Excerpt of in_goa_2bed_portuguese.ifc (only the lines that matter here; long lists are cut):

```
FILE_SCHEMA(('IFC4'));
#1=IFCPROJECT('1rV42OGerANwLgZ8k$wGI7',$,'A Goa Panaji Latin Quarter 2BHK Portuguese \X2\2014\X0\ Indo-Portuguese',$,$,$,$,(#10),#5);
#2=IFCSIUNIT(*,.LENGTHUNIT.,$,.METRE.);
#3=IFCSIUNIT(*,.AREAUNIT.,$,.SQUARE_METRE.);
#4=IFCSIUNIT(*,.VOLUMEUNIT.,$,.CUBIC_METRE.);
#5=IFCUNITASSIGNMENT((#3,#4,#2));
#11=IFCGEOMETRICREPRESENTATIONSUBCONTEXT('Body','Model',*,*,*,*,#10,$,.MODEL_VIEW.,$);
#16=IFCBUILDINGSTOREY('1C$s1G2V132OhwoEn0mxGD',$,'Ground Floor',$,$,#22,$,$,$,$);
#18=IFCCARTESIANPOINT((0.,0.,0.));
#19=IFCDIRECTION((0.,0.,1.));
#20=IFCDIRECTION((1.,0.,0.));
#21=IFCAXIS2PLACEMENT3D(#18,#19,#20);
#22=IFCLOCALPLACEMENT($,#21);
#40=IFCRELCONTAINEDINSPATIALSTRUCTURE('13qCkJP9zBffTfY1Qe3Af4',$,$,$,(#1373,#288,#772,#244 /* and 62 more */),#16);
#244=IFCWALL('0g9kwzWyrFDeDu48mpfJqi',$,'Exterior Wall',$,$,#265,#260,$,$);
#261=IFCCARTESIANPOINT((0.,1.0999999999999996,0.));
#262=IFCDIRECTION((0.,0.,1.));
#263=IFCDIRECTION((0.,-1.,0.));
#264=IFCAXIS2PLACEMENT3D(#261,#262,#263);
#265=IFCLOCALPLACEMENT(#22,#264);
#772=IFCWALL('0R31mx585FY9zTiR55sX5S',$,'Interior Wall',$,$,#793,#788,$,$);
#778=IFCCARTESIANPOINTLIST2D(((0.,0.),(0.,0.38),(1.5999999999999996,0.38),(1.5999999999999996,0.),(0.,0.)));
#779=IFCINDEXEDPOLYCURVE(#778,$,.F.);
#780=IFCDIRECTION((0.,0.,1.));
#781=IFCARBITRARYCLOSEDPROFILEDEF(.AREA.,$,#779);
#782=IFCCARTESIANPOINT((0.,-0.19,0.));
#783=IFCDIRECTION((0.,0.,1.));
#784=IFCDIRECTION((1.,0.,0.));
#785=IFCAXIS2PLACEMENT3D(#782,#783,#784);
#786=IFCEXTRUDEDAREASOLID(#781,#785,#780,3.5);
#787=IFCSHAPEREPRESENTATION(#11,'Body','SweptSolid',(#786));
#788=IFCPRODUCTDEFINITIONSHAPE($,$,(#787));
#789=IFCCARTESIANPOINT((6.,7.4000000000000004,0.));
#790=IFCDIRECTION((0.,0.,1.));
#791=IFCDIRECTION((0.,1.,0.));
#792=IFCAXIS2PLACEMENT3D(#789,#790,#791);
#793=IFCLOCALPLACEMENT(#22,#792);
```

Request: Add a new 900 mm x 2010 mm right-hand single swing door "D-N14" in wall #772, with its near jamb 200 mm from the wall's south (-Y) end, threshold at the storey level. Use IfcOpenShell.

```python
import numpy as np
import ifcopenshell
import ifcopenshell.api.feature
import ifcopenshell.api.geometry
import ifcopenshell.api.root
import ifcopenshell.api.spatial
import ifcopenshell.geom
import ifcopenshell.util.element
import ifcopenshell.util.placement
import ifcopenshell.util.representation
import ifcopenshell.util.shape
import ifcopenshell.util.unit

model = ifcopenshell.open("in_goa_2bed_portuguese.ifc")
unit_scale = ifcopenshell.util.unit.calculate_unit_scale(model)
settings = ifcopenshell.geom.settings()


def volume(element):
    """Net volume in cubic metres, openings subtracted."""
    shape = ifcopenshell.geom.create_shape(settings, element)
    return ifcopenshell.util.shape.get_volume(shape.geometry)


wall = model.by_id(772)
storey = ifcopenshell.util.element.get_container(wall, ifc_class="IfcBuildingStorey")
context = ifcopenshell.util.representation.get_context(model, "Model", "Body", "MODEL_VIEW")
before = volume(wall)

width, height, from_end, sill = 0.9, 2.01, 0.2, 0.0  # metres

# The wall runs along its own X axis, and the end named is its -X end.
wall_shape = ifcopenshell.geom.create_shape(settings, wall)
x, y, z = ifcopenshell.util.shape.get_vertices(wall_shape.geometry).T
start = x.min() + from_end
face, thickness = float(y.min()), float(y.max() - y.min())
wall_matrix = ifcopenshell.util.placement.get_local_placement(wall.ObjectPlacement)
level = ifcopenshell.util.placement.get_local_placement(storey.ObjectPlacement)[2, 3]


def in_wall(x, y):
    """Placement at x, y metres in the wall's axes, at sill height."""
    matrix = wall_matrix.copy()
    matrix[:, 3] = wall_matrix @ np.array([x / unit_scale, y / unit_scale, 0.0, 1.0])
    matrix[2, 3] = level + sill / unit_scale
    return matrix


# Opening: a box that overshoots both wall faces by 50 mm.
opening = ifcopenshell.api.root.create_entity(model, ifc_class="IfcOpeningElement", predefined_type="OPENING")
box = ifcopenshell.api.geometry.add_wall_representation(
    model, context=context, length=width, height=height, thickness=thickness + 0.1
)
ifcopenshell.api.geometry.assign_representation(model, product=opening, representation=box)
ifcopenshell.api.geometry.edit_object_placement(model, product=opening, matrix=in_wall(start, face - 0.05), is_si=False)
ifcopenshell.api.feature.add_feature(model, feature=opening, element=wall)

door = ifcopenshell.api.root.create_entity(model, ifc_class="IfcDoor", name="D-N14", predefined_type="DOOR")
door.OverallWidth, door.OverallHeight = width / unit_scale, height / unit_scale
door.OperationType = "SINGLE_SWING_RIGHT"
body = ifcopenshell.api.geometry.add_door_representation(
    model,
    context=context,
    overall_width=door.OverallWidth,
    overall_height=door.OverallHeight,
    operation_type="SINGLE_SWING_RIGHT",
    lining_properties={"LiningDepth": thickness / unit_scale, "ThresholdDepth": thickness / unit_scale},
)
ifcopenshell.api.geometry.assign_representation(model, product=door, representation=body)
ifcopenshell.api.spatial.assign_container(model, products=[door], relating_structure=storey)
ifcopenshell.api.feature.add_filling(model, opening=opening, element=door)

# The lining spans the wall, so the door starts at the wall face.
ifcopenshell.api.geometry.edit_object_placement(model, product=door, matrix=in_wall(start, face), is_si=False)

after = volume(wall)

print(f"wall volume {before:.3f} -> {after:.3f} m3")

model.write("in_goa_2bed_portuguese_rev.ifc")
```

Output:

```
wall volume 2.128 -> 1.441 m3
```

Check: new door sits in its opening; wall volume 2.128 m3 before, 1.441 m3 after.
